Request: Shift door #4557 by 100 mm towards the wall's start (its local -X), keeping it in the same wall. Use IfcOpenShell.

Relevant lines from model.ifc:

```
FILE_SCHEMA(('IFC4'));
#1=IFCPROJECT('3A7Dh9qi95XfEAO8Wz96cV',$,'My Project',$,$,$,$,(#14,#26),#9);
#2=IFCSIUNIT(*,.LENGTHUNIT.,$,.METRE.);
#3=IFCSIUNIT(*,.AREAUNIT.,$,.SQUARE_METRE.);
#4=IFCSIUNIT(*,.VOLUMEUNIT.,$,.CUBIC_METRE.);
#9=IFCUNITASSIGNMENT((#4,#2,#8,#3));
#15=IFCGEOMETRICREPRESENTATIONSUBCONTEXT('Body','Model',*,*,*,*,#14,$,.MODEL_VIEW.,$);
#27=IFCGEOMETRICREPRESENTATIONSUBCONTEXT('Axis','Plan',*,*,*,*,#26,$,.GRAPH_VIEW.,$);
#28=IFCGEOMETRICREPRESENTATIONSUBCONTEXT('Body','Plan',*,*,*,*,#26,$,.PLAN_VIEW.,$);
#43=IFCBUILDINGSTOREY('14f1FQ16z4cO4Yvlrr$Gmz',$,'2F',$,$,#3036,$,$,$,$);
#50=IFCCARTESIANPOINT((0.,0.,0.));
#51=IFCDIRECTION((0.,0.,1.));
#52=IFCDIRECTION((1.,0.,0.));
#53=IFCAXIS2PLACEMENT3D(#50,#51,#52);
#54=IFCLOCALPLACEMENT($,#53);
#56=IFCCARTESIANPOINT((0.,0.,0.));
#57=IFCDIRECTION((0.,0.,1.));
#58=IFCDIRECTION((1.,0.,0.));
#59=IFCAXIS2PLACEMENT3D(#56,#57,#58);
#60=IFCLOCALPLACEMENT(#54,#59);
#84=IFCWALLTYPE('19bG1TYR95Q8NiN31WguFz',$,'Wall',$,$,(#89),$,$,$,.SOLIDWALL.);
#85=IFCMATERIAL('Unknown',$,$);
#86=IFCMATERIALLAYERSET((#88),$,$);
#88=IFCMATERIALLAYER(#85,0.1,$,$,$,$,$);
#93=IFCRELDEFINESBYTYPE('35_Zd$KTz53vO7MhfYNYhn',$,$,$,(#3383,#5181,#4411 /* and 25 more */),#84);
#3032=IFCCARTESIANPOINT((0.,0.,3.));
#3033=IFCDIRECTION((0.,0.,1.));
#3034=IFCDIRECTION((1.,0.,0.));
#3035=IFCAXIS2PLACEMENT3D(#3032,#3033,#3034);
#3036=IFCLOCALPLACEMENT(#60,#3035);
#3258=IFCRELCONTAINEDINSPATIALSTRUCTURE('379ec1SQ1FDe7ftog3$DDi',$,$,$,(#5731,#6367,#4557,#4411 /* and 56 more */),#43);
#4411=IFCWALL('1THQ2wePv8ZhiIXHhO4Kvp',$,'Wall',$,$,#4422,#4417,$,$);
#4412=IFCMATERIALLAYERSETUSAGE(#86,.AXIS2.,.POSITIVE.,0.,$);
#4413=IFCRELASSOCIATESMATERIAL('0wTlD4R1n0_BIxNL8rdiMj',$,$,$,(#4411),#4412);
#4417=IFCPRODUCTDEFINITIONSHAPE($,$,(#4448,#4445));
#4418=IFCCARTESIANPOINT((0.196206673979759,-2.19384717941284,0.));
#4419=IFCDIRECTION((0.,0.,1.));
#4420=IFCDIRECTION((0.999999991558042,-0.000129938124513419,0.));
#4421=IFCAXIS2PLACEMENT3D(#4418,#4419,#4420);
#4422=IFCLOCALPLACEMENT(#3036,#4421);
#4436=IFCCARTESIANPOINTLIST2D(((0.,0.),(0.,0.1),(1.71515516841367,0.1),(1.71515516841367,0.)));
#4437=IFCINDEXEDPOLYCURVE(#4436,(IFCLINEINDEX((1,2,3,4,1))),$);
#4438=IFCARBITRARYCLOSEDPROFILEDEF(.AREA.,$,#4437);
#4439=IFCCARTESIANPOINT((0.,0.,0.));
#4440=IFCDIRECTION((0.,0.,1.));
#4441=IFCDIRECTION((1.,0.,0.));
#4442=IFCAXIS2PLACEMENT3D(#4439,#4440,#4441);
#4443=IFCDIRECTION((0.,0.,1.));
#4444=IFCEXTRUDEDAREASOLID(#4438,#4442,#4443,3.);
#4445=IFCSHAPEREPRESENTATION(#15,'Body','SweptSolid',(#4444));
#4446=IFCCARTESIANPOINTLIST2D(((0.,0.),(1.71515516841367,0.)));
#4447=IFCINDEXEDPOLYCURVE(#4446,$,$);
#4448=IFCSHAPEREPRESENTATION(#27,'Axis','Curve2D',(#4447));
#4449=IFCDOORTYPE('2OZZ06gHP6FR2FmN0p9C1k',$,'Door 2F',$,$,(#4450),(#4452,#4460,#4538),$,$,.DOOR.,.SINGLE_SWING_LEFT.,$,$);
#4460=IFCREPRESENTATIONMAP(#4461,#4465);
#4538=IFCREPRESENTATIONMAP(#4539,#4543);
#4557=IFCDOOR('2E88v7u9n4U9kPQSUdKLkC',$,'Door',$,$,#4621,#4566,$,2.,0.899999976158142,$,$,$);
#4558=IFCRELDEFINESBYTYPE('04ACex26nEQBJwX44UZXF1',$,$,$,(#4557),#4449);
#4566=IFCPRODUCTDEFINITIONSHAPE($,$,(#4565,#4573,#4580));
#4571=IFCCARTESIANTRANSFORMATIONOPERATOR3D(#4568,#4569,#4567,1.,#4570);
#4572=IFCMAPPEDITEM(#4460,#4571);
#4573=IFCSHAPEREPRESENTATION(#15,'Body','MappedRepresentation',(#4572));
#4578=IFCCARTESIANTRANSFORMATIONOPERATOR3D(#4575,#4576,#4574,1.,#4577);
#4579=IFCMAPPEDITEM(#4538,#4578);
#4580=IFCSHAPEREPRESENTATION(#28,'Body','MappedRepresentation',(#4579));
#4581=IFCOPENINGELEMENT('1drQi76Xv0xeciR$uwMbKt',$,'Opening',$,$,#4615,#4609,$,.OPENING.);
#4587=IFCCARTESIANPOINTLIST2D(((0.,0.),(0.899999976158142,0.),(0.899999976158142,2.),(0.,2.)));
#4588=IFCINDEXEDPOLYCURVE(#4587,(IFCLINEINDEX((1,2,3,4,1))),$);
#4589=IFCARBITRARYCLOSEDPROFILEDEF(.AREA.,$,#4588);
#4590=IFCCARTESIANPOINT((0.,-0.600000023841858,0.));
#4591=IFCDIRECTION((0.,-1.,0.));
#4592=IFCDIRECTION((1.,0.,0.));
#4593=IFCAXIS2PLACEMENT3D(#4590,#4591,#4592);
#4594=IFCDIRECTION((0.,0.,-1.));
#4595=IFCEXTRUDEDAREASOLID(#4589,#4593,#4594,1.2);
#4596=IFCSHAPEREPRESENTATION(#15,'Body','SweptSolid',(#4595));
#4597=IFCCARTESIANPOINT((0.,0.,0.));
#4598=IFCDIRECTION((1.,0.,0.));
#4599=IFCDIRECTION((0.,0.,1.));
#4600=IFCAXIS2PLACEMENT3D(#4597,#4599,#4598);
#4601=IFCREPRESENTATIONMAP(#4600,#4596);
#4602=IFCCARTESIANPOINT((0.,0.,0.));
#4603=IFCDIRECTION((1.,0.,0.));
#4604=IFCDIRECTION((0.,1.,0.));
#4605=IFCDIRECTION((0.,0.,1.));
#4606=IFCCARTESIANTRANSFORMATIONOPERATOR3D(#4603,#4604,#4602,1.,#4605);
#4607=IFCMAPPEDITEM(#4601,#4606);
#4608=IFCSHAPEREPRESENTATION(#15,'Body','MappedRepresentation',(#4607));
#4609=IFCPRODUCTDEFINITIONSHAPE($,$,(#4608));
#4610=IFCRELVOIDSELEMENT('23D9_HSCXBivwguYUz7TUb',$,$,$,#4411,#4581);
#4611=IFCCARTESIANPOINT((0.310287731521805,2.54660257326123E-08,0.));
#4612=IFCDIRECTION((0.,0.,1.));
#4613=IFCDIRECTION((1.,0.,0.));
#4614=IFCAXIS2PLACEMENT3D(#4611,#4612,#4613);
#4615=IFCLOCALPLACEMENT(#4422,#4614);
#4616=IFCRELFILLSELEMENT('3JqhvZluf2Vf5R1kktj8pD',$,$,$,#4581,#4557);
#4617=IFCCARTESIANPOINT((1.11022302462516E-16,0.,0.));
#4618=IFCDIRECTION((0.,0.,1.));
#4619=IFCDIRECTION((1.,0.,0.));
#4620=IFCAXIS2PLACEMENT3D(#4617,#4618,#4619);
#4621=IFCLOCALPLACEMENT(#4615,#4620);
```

```python
import ifcopenshell
import ifcopenshell.api.geometry
import ifcopenshell.util.placement
import ifcopenshell.util.unit

model = ifcopenshell.open("model.ifc")
unit_scale = ifcopenshell.util.unit.calculate_unit_scale(model)

door = model.by_id(4557)
opening = door.FillsVoids[0].RelatingOpeningElement
wall = opening.VoidsElements[0].RelatingBuildingElement

wall_matrix = ifcopenshell.util.placement.get_local_placement(wall.ObjectPlacement)
shift = wall_matrix[:3, 0] * -0.1 / unit_scale
before = ifcopenshell.util.placement.get_local_placement(door.ObjectPlacement)[:3, 3].copy()

# The door is placed relative to its opening, so it follows when the opening moves.
matrix = ifcopenshell.util.placement.get_local_placement(opening.ObjectPlacement)
matrix[:3, 3] += shift
ifcopenshell.api.geometry.edit_object_placement(
    model, product=opening, matrix=matrix, is_si=False, should_transform_children=True
)

after = ifcopenshell.util.placement.get_local_placement(door.ObjectPlacement)[:3, 3]
print("door moved by", (after - before).round(3) + 0.0)

model.write("model_rev.ifc")
```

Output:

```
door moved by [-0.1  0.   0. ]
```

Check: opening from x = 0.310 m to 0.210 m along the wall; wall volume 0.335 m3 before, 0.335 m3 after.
